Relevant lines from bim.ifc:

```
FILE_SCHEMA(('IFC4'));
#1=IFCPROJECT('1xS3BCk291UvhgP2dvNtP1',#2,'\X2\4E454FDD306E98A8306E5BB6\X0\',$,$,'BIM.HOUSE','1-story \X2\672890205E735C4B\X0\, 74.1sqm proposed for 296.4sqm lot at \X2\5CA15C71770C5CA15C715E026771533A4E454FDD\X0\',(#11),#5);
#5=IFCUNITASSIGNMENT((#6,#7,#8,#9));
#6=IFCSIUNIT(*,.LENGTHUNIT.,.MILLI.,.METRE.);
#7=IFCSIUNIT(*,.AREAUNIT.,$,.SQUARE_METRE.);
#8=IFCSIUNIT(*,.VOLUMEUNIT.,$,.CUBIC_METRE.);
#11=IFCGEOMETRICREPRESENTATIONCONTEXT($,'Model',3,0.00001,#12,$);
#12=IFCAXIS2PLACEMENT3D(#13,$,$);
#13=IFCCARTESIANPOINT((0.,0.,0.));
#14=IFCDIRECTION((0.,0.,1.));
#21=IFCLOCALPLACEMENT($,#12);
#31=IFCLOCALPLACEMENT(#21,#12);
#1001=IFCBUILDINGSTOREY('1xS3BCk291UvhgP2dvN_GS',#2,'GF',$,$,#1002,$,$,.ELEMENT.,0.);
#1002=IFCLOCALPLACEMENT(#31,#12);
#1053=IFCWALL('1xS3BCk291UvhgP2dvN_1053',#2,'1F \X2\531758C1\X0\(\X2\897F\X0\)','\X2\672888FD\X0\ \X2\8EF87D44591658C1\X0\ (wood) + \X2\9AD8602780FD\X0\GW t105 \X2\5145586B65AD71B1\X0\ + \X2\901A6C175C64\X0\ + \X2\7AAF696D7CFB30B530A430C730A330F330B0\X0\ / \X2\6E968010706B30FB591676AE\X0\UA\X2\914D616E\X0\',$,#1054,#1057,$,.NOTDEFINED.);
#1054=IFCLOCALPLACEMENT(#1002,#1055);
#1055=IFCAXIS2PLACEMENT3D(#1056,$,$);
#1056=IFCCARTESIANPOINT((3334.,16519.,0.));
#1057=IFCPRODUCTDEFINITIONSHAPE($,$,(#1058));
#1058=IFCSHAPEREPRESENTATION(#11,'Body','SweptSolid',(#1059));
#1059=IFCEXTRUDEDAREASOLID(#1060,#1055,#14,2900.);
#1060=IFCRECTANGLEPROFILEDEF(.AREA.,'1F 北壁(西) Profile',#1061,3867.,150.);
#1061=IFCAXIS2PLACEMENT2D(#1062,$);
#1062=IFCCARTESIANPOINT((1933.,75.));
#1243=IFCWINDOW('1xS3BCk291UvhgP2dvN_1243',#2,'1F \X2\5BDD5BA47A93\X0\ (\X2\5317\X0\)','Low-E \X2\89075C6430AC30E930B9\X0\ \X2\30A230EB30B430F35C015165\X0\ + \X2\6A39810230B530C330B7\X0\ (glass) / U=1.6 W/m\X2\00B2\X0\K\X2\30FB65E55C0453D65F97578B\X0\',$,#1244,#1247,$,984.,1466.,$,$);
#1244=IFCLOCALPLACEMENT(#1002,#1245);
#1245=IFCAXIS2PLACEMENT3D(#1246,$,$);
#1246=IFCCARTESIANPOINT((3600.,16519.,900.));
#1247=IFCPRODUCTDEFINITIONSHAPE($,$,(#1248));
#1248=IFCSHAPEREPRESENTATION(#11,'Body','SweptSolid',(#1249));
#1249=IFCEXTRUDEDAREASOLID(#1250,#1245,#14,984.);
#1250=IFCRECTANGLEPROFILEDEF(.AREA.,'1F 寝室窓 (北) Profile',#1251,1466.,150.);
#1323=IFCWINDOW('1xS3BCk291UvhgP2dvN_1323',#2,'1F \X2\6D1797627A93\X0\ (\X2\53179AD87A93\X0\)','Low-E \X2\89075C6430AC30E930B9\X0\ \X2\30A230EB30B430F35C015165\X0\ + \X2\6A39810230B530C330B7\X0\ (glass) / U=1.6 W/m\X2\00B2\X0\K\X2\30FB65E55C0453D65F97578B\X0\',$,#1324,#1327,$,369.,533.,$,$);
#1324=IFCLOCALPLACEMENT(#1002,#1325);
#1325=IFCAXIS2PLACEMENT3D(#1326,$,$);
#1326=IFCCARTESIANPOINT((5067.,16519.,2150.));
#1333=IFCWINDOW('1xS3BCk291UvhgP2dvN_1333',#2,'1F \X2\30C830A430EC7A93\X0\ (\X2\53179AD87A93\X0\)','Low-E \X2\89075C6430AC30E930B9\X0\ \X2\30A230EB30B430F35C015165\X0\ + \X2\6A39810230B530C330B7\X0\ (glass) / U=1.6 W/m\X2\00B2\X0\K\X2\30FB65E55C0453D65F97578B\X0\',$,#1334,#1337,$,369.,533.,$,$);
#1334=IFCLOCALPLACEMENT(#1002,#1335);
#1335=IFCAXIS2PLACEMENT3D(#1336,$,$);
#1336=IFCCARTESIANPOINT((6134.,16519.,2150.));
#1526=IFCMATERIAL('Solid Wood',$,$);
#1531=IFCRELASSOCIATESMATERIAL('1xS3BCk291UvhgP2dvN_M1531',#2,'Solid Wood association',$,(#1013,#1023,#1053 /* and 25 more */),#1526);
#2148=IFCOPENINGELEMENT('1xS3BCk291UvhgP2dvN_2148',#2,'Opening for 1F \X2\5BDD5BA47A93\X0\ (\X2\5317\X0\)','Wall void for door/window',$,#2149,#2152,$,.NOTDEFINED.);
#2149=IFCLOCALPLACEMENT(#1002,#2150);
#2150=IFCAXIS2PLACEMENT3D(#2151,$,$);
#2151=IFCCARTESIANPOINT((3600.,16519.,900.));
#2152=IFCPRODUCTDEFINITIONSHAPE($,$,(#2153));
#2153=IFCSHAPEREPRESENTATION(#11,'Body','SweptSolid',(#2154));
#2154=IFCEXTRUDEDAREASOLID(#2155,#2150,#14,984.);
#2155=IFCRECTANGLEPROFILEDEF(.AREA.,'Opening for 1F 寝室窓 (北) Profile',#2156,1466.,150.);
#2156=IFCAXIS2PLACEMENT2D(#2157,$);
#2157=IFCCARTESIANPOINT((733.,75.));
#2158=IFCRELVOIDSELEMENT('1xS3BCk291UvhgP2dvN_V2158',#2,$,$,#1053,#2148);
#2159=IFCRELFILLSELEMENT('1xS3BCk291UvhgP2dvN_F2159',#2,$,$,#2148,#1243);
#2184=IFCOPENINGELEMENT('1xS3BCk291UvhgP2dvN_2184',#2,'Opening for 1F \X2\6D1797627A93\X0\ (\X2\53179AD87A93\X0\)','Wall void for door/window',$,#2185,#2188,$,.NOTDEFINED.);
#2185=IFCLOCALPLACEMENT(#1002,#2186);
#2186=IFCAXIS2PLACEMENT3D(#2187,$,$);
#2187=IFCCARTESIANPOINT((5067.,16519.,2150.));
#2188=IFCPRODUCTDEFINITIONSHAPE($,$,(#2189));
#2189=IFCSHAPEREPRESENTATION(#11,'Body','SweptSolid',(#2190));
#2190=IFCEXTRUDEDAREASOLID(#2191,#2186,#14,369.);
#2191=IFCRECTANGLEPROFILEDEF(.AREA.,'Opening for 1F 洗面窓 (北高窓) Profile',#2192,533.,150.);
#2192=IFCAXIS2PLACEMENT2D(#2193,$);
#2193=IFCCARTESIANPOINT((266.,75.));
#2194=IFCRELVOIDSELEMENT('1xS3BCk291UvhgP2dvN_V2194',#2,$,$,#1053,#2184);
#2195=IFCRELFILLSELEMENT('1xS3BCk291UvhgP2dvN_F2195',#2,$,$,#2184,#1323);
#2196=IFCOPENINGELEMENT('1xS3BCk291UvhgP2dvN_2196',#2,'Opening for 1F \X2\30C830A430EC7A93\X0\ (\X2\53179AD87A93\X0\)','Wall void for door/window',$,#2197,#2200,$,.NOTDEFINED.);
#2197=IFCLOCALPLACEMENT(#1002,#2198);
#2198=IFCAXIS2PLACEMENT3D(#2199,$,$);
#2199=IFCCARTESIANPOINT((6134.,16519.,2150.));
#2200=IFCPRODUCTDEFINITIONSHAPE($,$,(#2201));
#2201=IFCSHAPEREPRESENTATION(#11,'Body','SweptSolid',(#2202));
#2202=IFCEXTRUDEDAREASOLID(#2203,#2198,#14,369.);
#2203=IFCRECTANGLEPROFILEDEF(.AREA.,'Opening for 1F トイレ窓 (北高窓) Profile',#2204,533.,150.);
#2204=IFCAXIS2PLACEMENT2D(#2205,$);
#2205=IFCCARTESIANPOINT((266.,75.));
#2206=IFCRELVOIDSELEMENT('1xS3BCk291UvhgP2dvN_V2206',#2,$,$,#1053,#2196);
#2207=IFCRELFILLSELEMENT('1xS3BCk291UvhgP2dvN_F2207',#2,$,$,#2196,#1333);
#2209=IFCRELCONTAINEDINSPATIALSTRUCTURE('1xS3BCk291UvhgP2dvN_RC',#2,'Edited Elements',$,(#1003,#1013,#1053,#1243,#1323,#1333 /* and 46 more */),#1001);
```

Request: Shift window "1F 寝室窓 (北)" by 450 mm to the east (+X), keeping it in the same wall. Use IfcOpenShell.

```python
import ifcopenshell
import ifcopenshell.api.geometry
import ifcopenshell.util.placement
import ifcopenshell.util.unit

model = ifcopenshell.open("bim.ifc")
unit_scale = ifcopenshell.util.unit.calculate_unit_scale(model)

window = model.by_guid("1xS3BCk291UvhgP2dvN_1243")
opening = window.FillsVoids[0].RelatingOpeningElement
wall = opening.VoidsElements[0].RelatingBuildingElement

wall_matrix = ifcopenshell.util.placement.get_local_placement(wall.ObjectPlacement)
shift = wall_matrix[:3, 0] * 0.45 / unit_scale
before = ifcopenshell.util.placement.get_local_placement(window.ObjectPlacement)[:3, 3].copy()

# The window is not placed relative to its opening, so move both.
for product in (opening, window):
    matrix = ifcopenshell.util.placement.get_local_placement(product.ObjectPlacement)
    matrix[:3, 3] += shift
    ifcopenshell.api.geometry.edit_object_placement(model, product=product, matrix=matrix, is_si=False)

after = ifcopenshell.util.placement.get_local_placement(window.ObjectPlacement)[:3, 3]
print("window moved by", (after - before).round(3) + 0.0)

model.write("bim_updated.ifc")
```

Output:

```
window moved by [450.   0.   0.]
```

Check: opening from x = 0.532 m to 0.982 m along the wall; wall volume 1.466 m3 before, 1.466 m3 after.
